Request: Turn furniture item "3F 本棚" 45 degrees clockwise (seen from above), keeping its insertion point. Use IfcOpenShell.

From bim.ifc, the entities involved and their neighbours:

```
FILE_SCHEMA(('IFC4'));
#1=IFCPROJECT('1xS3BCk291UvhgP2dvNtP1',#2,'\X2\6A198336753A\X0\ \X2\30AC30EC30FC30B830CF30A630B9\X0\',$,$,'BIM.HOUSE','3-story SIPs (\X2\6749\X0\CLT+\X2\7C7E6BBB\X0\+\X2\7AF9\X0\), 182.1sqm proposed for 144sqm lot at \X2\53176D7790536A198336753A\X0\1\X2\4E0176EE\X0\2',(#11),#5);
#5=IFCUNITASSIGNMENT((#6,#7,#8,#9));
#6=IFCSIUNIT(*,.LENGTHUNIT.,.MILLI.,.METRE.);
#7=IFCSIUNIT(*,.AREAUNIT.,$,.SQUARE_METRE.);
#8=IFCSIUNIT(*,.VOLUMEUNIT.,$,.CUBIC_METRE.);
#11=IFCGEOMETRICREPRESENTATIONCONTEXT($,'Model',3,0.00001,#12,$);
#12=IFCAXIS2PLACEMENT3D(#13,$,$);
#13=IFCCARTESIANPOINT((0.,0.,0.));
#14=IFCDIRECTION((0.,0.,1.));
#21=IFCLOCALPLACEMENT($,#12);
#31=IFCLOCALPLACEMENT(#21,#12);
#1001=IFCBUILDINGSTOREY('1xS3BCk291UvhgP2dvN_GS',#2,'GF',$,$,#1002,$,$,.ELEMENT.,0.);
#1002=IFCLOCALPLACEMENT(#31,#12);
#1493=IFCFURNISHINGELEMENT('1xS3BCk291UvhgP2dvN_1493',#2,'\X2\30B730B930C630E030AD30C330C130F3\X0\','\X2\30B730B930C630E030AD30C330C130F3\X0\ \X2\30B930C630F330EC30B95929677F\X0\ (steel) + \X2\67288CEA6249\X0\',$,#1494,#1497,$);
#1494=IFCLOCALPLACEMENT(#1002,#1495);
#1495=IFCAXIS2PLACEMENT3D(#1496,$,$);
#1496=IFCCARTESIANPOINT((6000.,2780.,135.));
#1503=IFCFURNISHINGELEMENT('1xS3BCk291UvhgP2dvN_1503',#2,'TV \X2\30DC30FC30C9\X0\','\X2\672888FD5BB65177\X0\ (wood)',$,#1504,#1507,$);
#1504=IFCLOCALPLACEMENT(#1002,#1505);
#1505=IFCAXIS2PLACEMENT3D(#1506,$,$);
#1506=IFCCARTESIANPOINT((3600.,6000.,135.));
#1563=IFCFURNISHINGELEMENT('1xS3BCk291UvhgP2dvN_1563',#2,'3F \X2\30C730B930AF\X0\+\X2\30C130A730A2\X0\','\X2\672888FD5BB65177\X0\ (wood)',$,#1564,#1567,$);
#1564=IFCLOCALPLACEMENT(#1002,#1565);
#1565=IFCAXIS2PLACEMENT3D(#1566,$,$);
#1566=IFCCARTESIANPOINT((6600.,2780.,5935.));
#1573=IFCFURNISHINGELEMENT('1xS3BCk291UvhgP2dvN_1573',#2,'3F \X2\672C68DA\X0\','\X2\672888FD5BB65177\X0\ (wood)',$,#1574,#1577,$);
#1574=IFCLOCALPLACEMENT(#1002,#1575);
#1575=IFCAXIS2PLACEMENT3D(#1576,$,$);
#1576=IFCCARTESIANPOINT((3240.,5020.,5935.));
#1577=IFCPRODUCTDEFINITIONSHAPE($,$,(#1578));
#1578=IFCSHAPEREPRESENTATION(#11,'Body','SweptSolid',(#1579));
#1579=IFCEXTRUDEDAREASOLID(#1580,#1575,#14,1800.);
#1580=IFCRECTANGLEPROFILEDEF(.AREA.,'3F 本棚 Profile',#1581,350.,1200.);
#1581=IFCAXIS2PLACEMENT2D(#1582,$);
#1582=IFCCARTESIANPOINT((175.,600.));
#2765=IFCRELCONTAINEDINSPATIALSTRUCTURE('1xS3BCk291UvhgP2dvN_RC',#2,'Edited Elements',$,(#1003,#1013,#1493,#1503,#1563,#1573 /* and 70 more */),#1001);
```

```python
import ifcopenshell
import ifcopenshell.api.geometry
import ifcopenshell.util.placement

model = ifcopenshell.open("bim.ifc")

item = model.by_id(1573)
matrix = ifcopenshell.util.placement.get_local_placement(item.ObjectPlacement)
matrix = matrix @ ifcopenshell.util.placement.rotation(-45, "Z")
ifcopenshell.api.geometry.edit_object_placement(model, product=item, matrix=matrix, is_si=False)

print(ifcopenshell.util.placement.get_local_placement(item.ObjectPlacement).round(3) + 0.0)

model.write("bim_updated.ifc")
```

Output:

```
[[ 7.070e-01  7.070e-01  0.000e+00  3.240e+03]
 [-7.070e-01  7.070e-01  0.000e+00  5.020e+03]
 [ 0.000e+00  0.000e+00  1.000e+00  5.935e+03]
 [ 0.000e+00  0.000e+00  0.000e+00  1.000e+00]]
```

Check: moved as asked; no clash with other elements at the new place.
